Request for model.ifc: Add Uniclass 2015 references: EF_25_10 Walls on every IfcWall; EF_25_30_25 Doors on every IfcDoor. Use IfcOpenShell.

First a look at what the model holds.

```python
import ifcopenshell

model = ifcopenshell.open("model.ifc")
print(model.schema)
print("classifications:", [c.Name for c in model.by_type("IfcClassification")])
for ifc_class in ("IfcDoor", "IfcRoof", "IfcStair", "IfcWall", "IfcWindow"):
    print(ifc_class, len(model.by_type(ifc_class)))
```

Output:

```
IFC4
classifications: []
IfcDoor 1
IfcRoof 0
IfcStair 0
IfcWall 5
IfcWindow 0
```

```python
import ifcopenshell
import ifcopenshell.api.classification

model = ifcopenshell.open("model.ifc")

system = ifcopenshell.api.classification.add_classification(model, classification="Uniclass 2015")

codes = {
    "IfcWall": ("EF_25_10", "Walls"),
    "IfcDoor": ("EF_25_30_25", "Doors"),
}
for ifc_class, (code, name) in codes.items():
    products = model.by_type(ifc_class)
    ifcopenshell.api.classification.add_reference(
        model, products=products, classification=system, identification=code, name=name
    )
    print(code, len(products))

model.write("model_v2.ifc")
```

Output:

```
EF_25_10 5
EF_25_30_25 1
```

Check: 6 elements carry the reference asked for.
